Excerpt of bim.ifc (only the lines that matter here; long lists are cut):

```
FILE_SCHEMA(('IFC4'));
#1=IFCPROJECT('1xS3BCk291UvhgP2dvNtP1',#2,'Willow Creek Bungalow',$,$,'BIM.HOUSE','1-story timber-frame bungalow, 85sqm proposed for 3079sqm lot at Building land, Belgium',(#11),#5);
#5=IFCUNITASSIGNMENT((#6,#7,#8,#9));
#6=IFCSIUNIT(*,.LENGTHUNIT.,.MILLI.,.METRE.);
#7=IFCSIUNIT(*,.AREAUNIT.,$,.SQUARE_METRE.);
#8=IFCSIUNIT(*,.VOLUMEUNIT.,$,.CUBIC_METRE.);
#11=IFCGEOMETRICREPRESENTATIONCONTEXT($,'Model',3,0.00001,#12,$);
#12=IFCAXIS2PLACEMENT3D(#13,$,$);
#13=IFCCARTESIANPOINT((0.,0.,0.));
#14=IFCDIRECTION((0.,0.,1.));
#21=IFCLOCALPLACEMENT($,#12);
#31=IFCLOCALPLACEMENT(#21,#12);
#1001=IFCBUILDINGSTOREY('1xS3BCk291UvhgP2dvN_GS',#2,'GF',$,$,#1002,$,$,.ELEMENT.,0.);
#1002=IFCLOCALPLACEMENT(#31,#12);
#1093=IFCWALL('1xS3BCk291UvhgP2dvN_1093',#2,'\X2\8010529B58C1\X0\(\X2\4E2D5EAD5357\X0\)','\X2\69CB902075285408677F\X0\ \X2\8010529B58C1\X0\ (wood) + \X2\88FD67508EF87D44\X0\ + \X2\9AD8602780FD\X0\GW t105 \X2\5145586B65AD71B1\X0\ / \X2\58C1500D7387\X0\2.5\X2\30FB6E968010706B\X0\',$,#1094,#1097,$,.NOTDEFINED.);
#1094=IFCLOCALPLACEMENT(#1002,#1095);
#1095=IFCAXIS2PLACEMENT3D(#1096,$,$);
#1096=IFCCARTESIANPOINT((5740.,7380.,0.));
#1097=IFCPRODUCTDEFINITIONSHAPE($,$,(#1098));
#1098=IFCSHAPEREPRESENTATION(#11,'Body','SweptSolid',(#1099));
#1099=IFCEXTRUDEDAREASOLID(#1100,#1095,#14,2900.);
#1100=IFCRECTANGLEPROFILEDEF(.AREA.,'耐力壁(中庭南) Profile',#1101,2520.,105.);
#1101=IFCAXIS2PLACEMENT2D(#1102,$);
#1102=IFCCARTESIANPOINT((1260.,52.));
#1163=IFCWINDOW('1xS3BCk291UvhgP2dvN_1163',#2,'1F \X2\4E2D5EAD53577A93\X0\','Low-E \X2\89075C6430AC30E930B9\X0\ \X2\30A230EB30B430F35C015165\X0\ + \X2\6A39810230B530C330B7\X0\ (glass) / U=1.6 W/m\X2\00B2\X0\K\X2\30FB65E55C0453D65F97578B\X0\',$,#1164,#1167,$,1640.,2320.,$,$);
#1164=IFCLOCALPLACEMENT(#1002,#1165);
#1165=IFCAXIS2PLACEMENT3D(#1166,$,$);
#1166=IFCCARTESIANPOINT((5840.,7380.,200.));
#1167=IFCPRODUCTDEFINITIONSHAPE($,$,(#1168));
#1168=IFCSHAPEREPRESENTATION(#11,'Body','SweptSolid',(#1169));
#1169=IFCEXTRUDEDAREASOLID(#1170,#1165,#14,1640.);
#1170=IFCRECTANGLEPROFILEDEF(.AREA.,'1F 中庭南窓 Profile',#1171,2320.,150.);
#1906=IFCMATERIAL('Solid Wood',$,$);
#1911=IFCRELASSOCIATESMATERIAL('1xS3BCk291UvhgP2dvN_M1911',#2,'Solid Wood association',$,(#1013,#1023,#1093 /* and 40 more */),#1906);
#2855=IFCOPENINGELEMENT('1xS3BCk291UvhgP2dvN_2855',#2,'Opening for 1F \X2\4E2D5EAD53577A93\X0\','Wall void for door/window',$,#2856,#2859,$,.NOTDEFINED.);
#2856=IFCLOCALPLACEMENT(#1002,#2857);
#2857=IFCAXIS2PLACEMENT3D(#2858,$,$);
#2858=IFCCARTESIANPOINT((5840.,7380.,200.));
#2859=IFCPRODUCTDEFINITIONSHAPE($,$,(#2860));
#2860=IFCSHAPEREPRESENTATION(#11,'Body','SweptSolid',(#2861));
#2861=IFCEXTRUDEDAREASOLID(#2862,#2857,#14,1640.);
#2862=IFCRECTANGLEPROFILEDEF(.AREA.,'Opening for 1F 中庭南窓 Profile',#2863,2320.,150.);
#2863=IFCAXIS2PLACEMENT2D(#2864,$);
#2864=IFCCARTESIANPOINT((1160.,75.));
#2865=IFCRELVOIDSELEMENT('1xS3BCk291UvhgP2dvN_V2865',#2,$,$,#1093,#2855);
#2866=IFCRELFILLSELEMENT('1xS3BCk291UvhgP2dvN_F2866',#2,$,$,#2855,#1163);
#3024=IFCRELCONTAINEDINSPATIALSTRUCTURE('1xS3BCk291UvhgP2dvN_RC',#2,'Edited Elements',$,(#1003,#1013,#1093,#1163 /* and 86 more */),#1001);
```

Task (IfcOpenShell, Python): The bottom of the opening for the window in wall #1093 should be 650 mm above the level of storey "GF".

```python
import numpy as np
import ifcopenshell
import ifcopenshell.api.geometry
import ifcopenshell.geom
import ifcopenshell.util.element
import ifcopenshell.util.placement
import ifcopenshell.util.shape
import ifcopenshell.util.unit

model = ifcopenshell.open("bim.ifc")
unit_scale = ifcopenshell.util.unit.calculate_unit_scale(model)

window = model.by_guid("1xS3BCk291UvhgP2dvN_1163")
opening = window.FillsVoids[0].RelatingOpeningElement
storey = ifcopenshell.util.element.get_container(window, ifc_class="IfcBuildingStorey")
level = ifcopenshell.util.placement.get_local_placement(storey.ObjectPlacement)[2, 3]

# The opening's origin need not be at the sill, so measure its lowest point.
shape = ifcopenshell.geom.create_shape(ifcopenshell.geom.settings(), opening)
bottom = ifcopenshell.util.shape.get_shape_bottom_elevation(shape, shape.geometry) / unit_scale
dz = level + 0.65 / unit_scale - bottom

shift = np.array([0.0, 0.0, dz])
# The window is not placed relative to its opening, so move both.
for product in (opening, window):
    matrix = ifcopenshell.util.placement.get_local_placement(product.ObjectPlacement)
    matrix[:3, 3] += shift
    ifcopenshell.api.geometry.edit_object_placement(model, product=product, matrix=matrix, is_si=False)

print(f"moved by {dz * unit_scale:+.3f} m")

model.write("bim_updated.ifc")
```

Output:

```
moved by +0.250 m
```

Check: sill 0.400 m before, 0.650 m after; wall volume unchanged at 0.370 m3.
